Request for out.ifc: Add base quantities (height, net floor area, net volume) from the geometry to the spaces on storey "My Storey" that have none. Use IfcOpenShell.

First a look at what the model holds.

```python
import ifcopenshell
import ifcopenshell.util.element
import ifcopenshell.util.unit

model = ifcopenshell.open("out.ifc")
print(model.schema)
for unit_type in ("LENGTHUNIT", "AREAUNIT", "VOLUMEUNIT"):
    print(unit_type, ifcopenshell.util.unit.calculate_unit_scale(model, unit_type))
storey = next(s for s in model.by_type("IfcBuildingStorey") if s.Name == "My Storey")
spaces = [e for e in ifcopenshell.util.element.get_decomposition(storey) if e.is_a("IfcSpace")]
for e in sorted(spaces, key=lambda e: e.id()):
    print(e.id(), e.is_a(), e.Name, list(ifcopenshell.util.element.get_psets(e, qtos_only=True)), sep=" | ")
```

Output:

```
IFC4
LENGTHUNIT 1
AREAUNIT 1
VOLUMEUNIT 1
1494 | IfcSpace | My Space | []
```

```python
import ifcopenshell
import ifcopenshell.api.pset
import ifcopenshell.geom
import ifcopenshell.util.element
import ifcopenshell.util.shape
import ifcopenshell.util.unit

model = ifcopenshell.open("out.ifc")
unit_scale = ifcopenshell.util.unit.calculate_unit_scale(model)
area_scale = ifcopenshell.util.unit.calculate_unit_scale(model, "AREAUNIT")
volume_scale = ifcopenshell.util.unit.calculate_unit_scale(model, "VOLUMEUNIT")
settings = ifcopenshell.geom.settings()

storey = next(s for s in model.by_type("IfcBuildingStorey") if s.Name == "My Storey")
spaces = [e for e in ifcopenshell.util.element.get_decomposition(storey) if e.is_a("IfcSpace")]

for e in sorted(spaces, key=lambda e: e.id()):
    if ifcopenshell.util.element.get_psets(e, qtos_only=True, should_inherit=False):
        continue
    # Geometry comes back in metres, in the element's own axes.
    shape = ifcopenshell.geom.create_shape(settings, e)
    values = {
        "Height": ifcopenshell.util.shape.get_z(shape.geometry) / unit_scale,
        "NetFloorArea": ifcopenshell.util.shape.get_footprint_area(shape.geometry) / area_scale,
        "NetVolume": ifcopenshell.util.shape.get_volume(shape.geometry) / volume_scale,
    }
    qto = ifcopenshell.api.pset.add_qto(model, product=e, name="Qto_SpaceBaseQuantities")
    ifcopenshell.api.pset.edit_qto(model, qto=qto, properties=values)
    print(e.id(), {k: round(v, 3) for k, v in values.items()})

model.write("out_v2.ifc")
```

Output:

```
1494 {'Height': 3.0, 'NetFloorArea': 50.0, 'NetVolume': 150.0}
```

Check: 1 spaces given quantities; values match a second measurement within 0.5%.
